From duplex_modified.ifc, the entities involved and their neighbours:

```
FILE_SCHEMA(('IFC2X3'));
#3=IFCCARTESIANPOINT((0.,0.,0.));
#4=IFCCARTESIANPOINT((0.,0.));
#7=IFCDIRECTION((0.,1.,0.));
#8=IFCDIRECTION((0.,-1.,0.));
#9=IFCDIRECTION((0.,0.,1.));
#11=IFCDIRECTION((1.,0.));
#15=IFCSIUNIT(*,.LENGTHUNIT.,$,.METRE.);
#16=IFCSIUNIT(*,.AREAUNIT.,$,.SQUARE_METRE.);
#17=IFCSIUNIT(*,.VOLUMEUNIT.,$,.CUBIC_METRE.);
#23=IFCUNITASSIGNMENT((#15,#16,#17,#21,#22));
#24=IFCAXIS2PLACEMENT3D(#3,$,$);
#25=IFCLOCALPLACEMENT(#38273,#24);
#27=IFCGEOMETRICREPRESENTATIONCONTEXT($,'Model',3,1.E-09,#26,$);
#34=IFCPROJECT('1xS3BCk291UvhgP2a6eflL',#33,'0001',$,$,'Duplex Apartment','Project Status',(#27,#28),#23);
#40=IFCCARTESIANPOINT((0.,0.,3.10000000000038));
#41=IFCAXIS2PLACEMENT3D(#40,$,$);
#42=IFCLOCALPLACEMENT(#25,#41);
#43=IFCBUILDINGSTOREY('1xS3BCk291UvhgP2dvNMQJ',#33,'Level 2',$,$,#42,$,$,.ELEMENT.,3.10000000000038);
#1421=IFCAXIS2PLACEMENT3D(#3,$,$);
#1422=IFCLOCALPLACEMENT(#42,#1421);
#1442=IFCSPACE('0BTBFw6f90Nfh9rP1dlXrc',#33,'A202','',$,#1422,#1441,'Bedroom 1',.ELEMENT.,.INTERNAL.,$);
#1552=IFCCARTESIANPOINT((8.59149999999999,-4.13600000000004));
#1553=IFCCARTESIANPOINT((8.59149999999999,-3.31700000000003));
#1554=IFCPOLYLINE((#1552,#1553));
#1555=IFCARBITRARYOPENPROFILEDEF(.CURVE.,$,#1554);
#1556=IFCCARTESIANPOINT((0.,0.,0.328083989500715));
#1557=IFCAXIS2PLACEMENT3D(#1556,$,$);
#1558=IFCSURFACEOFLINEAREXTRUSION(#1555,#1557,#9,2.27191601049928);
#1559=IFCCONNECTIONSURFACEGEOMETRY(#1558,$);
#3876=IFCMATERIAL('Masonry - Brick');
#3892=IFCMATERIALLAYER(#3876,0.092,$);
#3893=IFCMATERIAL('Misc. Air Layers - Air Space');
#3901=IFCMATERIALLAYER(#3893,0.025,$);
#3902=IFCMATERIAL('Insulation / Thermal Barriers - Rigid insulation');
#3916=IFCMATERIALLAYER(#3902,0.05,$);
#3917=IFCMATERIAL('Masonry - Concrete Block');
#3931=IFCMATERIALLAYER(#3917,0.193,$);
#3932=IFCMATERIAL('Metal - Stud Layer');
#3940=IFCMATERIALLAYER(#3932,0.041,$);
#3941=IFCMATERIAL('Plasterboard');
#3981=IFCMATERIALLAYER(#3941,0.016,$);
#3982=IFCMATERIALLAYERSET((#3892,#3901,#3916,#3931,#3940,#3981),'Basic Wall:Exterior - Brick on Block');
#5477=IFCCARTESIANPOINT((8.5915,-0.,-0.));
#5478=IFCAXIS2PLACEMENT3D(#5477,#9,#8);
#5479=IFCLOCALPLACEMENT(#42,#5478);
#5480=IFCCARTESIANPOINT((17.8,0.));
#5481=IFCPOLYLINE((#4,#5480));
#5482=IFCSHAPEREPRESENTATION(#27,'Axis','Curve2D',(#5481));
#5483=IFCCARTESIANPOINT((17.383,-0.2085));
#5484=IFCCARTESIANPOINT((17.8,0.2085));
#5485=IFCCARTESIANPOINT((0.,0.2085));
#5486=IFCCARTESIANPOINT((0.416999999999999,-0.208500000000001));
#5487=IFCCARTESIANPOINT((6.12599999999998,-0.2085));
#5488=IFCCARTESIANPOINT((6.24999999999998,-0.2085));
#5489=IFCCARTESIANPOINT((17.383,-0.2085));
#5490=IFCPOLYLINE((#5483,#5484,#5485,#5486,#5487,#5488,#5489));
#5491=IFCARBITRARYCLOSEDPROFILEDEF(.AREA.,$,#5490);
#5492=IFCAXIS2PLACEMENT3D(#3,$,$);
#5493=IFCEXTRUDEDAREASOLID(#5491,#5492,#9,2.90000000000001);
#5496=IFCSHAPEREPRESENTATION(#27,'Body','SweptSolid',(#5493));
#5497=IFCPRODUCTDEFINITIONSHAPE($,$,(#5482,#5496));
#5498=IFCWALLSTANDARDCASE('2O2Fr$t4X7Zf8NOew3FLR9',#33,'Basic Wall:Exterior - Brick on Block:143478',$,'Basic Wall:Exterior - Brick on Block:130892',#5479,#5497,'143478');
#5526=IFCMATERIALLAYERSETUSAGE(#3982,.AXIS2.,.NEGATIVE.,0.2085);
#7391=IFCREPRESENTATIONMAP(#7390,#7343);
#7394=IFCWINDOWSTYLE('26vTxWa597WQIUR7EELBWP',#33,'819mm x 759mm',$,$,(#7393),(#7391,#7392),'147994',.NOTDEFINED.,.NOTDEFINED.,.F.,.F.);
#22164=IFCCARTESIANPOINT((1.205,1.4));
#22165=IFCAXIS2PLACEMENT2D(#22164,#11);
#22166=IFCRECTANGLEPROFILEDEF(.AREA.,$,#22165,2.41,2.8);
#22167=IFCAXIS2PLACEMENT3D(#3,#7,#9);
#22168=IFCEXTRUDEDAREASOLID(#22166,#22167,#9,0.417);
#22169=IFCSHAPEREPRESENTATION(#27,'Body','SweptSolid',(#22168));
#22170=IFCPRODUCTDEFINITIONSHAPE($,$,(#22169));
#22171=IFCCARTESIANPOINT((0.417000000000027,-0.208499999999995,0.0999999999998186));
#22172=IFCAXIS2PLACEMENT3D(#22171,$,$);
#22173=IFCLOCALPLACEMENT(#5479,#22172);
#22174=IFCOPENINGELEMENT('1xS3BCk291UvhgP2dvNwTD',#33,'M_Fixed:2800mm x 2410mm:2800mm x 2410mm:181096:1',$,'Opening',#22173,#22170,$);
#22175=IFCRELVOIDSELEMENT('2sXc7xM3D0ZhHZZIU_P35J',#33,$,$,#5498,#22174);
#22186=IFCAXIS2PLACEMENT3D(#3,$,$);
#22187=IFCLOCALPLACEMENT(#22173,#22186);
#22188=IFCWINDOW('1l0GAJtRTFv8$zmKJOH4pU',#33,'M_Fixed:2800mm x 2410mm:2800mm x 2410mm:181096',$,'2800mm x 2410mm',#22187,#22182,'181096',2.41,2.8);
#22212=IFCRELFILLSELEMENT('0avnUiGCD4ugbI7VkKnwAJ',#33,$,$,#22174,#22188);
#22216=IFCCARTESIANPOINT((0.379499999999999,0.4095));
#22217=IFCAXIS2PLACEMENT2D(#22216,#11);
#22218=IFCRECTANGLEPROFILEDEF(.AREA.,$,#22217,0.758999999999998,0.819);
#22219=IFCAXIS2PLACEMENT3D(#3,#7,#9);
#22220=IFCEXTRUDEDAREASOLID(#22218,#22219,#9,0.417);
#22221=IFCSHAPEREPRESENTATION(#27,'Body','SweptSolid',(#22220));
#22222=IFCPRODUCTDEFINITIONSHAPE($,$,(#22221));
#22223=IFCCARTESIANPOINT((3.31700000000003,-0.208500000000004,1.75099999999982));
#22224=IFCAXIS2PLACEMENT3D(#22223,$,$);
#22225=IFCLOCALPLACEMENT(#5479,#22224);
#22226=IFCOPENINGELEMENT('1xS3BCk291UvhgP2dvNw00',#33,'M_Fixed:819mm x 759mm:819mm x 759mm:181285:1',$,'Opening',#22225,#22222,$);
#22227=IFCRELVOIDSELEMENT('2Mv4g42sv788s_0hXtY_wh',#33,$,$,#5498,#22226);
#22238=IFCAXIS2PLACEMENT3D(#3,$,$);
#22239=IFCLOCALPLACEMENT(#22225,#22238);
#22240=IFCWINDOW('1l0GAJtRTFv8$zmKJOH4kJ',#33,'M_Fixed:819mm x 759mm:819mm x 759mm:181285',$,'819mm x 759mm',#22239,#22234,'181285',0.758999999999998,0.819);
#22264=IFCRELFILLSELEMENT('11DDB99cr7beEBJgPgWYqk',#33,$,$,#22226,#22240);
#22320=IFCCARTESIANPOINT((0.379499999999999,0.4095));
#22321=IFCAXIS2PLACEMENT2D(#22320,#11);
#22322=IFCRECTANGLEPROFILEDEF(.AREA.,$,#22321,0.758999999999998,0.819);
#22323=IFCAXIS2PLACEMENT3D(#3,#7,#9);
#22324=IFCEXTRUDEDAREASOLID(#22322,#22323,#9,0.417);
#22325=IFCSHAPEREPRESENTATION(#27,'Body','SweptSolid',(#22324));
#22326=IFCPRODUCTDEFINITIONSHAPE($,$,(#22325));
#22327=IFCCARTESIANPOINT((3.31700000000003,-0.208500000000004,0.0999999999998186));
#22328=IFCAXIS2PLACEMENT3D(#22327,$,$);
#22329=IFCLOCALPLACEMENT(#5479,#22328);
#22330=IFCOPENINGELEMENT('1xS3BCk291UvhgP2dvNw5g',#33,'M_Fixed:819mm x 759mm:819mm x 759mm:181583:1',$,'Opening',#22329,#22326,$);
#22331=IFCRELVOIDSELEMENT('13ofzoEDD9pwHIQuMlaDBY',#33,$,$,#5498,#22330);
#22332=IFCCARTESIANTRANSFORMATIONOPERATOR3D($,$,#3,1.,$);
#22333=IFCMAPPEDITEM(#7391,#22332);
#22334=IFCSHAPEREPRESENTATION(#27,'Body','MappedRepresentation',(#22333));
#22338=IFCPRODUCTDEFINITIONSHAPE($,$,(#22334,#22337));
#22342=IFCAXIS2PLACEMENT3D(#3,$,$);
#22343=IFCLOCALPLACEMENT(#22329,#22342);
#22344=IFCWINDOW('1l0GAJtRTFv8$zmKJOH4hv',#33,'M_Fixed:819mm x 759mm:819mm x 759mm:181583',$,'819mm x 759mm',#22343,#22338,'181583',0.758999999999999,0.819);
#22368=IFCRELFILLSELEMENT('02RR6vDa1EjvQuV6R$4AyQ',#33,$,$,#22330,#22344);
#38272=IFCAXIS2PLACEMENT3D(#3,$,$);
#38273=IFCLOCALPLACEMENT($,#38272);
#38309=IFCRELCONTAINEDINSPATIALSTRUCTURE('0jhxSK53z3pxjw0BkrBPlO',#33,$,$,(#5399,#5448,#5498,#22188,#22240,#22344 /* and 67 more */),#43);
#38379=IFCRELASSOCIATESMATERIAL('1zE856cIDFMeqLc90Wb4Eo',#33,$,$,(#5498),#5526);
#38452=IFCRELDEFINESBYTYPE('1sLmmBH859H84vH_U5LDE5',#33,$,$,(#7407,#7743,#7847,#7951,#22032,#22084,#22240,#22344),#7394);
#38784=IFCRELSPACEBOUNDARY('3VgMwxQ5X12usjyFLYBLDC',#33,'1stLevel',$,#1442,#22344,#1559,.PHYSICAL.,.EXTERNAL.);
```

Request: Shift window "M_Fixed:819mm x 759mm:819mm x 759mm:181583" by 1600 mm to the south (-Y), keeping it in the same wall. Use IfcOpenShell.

```python
import numpy as np
import ifcopenshell
import ifcopenshell.api.geometry
import ifcopenshell.util.placement

model = ifcopenshell.open("duplex_modified.ifc")

window = model.by_id(22344)
opening = window.FillsVoids[0].RelatingOpeningElement
wall = opening.VoidsElements[0].RelatingBuildingElement

wall_matrix = ifcopenshell.util.placement.get_local_placement(wall.ObjectPlacement)
shift = wall_matrix[:3, 0] * 1.6
before = ifcopenshell.util.placement.get_local_placement(window.ObjectPlacement)[:3, 3].copy()

# The window is placed relative to its opening, so it follows when the opening moves.
matrix = ifcopenshell.util.placement.get_local_placement(opening.ObjectPlacement)
matrix[:3, 3] += shift
ifcopenshell.api.geometry.edit_object_placement(
    model, product=opening, matrix=matrix, is_si=False, should_transform_children=True
)

# Space boundary surfaces are stored in each space's coordinates; move them too.
for rel in window.ProvidesBoundaries:
    if not rel.ConnectionGeometry:
        continue
    surface = rel.ConnectionGeometry.SurfaceOnRelatingElement
    space_matrix = ifcopenshell.util.placement.get_local_placement(rel.RelatingSpace.ObjectPlacement)
    point = np.array(surface.Position.Location.Coordinates) + space_matrix[:3, :3].T @ shift
    surface.Position = model.createIfcAxis2Placement3D(
        model.createIfcCartesianPoint(point.tolist()), surface.Position.Axis, surface.Position.RefDirection
    )

after = ifcopenshell.util.placement.get_local_placement(window.ObjectPlacement)[:3, 3]
print("window moved by", (after - before).round(3) + 0.0)

model.write("duplex_modified_updated.ifc")
```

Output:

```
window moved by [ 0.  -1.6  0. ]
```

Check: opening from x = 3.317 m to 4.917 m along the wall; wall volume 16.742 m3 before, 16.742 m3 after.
